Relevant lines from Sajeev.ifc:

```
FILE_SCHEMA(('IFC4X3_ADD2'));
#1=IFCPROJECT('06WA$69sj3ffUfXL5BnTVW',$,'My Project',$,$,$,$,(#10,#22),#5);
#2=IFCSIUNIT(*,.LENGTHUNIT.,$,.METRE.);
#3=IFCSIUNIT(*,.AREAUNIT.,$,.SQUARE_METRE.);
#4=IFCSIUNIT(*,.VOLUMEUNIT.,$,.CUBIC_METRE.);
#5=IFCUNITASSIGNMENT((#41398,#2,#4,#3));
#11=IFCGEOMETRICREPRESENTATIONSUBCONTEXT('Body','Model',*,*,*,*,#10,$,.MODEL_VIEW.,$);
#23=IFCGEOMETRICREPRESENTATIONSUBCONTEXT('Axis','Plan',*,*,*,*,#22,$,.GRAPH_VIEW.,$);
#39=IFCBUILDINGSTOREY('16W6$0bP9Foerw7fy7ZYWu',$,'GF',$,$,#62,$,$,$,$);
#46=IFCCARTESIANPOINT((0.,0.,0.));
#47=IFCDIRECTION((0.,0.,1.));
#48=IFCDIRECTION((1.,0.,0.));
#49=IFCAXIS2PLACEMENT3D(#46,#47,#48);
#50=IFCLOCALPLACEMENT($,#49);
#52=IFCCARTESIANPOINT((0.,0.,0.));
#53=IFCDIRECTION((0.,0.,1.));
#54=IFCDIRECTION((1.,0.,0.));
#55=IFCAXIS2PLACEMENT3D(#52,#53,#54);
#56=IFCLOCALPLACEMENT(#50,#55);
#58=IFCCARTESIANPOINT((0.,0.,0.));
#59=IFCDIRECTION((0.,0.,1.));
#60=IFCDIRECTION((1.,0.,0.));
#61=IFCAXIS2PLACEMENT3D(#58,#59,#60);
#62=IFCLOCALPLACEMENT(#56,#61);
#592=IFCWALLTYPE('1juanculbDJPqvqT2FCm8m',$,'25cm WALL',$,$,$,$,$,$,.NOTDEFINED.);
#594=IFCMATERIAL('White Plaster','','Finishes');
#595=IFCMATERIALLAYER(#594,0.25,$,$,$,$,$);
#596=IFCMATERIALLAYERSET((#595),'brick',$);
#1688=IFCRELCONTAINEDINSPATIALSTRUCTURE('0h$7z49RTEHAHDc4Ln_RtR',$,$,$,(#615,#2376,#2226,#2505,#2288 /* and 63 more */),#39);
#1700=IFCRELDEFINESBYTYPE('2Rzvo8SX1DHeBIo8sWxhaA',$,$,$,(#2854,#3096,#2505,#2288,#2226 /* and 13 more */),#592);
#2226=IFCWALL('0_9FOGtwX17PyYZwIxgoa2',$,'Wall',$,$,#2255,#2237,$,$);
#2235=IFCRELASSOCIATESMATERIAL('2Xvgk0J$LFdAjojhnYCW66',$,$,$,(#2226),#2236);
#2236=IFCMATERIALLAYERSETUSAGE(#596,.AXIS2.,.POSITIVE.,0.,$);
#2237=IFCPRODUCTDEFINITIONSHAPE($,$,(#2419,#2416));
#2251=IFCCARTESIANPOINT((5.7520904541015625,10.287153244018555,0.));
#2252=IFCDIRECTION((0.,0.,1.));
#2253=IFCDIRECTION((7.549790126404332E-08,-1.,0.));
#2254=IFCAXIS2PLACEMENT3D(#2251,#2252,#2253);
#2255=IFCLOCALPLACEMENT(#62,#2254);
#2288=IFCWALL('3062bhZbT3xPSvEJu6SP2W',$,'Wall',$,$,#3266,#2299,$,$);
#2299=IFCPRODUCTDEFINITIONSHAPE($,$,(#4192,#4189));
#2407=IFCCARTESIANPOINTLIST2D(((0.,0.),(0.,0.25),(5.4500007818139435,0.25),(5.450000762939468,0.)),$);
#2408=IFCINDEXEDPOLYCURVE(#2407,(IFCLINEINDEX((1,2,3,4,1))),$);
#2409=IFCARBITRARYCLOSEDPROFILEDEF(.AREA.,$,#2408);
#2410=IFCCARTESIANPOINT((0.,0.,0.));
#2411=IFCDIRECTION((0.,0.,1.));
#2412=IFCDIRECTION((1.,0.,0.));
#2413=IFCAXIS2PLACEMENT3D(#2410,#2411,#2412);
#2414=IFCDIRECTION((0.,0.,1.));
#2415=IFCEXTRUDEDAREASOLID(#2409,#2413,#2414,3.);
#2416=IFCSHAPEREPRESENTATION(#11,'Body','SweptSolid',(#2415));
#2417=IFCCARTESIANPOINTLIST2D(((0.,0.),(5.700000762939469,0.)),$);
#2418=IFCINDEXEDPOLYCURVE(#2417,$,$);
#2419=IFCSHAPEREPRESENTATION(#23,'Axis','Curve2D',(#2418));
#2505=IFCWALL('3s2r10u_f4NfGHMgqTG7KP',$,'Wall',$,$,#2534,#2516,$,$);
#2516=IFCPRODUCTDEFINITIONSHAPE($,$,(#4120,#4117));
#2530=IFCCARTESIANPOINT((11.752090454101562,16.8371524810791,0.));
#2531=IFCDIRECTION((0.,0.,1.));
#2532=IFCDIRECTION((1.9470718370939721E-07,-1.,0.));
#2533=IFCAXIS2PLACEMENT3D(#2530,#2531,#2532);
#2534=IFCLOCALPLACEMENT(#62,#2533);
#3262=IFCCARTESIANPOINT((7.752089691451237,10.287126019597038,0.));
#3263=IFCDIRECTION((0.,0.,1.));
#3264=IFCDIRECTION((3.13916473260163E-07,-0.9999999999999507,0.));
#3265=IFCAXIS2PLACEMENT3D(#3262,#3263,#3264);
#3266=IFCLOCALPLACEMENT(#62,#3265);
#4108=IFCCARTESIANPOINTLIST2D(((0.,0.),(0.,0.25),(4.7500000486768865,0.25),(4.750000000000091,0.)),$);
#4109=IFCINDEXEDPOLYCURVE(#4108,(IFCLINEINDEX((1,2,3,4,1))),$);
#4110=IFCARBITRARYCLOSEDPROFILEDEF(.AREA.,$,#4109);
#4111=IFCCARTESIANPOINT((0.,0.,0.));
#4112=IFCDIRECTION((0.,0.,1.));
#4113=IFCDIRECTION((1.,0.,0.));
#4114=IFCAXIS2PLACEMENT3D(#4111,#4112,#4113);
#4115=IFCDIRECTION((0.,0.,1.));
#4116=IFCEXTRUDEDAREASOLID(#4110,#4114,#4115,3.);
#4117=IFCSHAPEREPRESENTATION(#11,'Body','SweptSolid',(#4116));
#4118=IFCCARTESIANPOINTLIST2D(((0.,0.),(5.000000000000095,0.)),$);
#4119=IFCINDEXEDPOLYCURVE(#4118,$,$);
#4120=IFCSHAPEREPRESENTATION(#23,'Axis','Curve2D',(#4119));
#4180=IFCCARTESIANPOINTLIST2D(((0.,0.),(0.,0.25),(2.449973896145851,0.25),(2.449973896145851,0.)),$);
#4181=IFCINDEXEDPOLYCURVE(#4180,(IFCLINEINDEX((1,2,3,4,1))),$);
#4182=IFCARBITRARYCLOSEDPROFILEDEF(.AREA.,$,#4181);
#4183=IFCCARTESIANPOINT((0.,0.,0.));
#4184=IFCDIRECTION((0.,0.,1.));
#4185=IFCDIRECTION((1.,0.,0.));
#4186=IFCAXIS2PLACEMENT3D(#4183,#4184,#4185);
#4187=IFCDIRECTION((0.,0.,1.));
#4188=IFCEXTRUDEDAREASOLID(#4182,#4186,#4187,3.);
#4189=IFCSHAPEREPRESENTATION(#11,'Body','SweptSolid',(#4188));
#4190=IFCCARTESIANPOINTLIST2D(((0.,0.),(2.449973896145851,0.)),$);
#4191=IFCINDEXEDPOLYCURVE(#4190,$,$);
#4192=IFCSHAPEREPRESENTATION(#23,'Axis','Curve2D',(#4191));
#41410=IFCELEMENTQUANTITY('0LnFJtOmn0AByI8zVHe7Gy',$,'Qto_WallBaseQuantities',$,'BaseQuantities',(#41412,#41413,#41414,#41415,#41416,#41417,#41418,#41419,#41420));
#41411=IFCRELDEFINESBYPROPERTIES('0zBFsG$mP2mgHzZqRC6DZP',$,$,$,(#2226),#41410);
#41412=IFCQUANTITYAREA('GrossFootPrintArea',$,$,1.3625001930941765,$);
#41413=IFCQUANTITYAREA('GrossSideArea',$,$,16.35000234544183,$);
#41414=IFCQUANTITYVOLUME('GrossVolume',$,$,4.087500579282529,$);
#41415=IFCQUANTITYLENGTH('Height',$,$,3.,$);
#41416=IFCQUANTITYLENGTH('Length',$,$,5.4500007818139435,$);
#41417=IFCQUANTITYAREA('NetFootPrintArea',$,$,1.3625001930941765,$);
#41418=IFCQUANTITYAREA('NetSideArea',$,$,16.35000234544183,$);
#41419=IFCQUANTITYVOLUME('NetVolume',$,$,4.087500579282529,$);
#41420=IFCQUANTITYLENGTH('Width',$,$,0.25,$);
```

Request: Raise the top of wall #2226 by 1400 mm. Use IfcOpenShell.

```python
import ifcopenshell
import ifcopenshell.api.pset
import ifcopenshell.geom
import ifcopenshell.util.element
import ifcopenshell.util.representation
import ifcopenshell.util.shape
import ifcopenshell.util.unit

model = ifcopenshell.open("Sajeev.ifc")
unit_scale = ifcopenshell.util.unit.calculate_unit_scale(model)
area_scale = ifcopenshell.util.unit.calculate_unit_scale(model, "AREAUNIT")
volume_scale = ifcopenshell.util.unit.calculate_unit_scale(model, "VOLUMEUNIT")
settings = ifcopenshell.geom.settings()


def volume(element):
    """Net volume in cubic metres, openings subtracted."""
    shape = ifcopenshell.geom.create_shape(settings, element)
    return ifcopenshell.util.shape.get_volume(shape.geometry)


wall = model.by_guid("0_9FOGtwX17PyYZwIxgoa2")
before = volume(wall)

body = ifcopenshell.util.representation.get_representation(wall, "Model", "Body")
solid = body.Items[0]
old_height = solid.Depth
solid.Depth += 1.4 / unit_scale
after = volume(wall)
thickness = 0.25  # wall thickness in metres

# Update the stored height, areas and volumes.
qto = model.by_id(ifcopenshell.util.element.get_pset(wall, "Qto_WallBaseQuantities", should_inherit=False)["id"])
ifcopenshell.api.pset.edit_qto(model, qto=qto, properties={
    "GrossSideArea": ifcopenshell.util.element.get_pset(wall, "Qto_WallBaseQuantities", "GrossSideArea") * solid.Depth / old_height,
    "GrossVolume": ifcopenshell.util.element.get_pset(wall, "Qto_WallBaseQuantities", "GrossVolume") * solid.Depth / old_height,
    "Height": solid.Depth,
    "NetSideArea": after / thickness / area_scale,
    "NetVolume": after / volume_scale,
})

print(f"height {old_height:g} -> {solid.Depth:g}, volume {before:.3f} -> {after:.3f} m3")

model.write("Sajeev_updated.ifc")
```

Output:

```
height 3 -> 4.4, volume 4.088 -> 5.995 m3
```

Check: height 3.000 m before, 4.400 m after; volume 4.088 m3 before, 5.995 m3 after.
